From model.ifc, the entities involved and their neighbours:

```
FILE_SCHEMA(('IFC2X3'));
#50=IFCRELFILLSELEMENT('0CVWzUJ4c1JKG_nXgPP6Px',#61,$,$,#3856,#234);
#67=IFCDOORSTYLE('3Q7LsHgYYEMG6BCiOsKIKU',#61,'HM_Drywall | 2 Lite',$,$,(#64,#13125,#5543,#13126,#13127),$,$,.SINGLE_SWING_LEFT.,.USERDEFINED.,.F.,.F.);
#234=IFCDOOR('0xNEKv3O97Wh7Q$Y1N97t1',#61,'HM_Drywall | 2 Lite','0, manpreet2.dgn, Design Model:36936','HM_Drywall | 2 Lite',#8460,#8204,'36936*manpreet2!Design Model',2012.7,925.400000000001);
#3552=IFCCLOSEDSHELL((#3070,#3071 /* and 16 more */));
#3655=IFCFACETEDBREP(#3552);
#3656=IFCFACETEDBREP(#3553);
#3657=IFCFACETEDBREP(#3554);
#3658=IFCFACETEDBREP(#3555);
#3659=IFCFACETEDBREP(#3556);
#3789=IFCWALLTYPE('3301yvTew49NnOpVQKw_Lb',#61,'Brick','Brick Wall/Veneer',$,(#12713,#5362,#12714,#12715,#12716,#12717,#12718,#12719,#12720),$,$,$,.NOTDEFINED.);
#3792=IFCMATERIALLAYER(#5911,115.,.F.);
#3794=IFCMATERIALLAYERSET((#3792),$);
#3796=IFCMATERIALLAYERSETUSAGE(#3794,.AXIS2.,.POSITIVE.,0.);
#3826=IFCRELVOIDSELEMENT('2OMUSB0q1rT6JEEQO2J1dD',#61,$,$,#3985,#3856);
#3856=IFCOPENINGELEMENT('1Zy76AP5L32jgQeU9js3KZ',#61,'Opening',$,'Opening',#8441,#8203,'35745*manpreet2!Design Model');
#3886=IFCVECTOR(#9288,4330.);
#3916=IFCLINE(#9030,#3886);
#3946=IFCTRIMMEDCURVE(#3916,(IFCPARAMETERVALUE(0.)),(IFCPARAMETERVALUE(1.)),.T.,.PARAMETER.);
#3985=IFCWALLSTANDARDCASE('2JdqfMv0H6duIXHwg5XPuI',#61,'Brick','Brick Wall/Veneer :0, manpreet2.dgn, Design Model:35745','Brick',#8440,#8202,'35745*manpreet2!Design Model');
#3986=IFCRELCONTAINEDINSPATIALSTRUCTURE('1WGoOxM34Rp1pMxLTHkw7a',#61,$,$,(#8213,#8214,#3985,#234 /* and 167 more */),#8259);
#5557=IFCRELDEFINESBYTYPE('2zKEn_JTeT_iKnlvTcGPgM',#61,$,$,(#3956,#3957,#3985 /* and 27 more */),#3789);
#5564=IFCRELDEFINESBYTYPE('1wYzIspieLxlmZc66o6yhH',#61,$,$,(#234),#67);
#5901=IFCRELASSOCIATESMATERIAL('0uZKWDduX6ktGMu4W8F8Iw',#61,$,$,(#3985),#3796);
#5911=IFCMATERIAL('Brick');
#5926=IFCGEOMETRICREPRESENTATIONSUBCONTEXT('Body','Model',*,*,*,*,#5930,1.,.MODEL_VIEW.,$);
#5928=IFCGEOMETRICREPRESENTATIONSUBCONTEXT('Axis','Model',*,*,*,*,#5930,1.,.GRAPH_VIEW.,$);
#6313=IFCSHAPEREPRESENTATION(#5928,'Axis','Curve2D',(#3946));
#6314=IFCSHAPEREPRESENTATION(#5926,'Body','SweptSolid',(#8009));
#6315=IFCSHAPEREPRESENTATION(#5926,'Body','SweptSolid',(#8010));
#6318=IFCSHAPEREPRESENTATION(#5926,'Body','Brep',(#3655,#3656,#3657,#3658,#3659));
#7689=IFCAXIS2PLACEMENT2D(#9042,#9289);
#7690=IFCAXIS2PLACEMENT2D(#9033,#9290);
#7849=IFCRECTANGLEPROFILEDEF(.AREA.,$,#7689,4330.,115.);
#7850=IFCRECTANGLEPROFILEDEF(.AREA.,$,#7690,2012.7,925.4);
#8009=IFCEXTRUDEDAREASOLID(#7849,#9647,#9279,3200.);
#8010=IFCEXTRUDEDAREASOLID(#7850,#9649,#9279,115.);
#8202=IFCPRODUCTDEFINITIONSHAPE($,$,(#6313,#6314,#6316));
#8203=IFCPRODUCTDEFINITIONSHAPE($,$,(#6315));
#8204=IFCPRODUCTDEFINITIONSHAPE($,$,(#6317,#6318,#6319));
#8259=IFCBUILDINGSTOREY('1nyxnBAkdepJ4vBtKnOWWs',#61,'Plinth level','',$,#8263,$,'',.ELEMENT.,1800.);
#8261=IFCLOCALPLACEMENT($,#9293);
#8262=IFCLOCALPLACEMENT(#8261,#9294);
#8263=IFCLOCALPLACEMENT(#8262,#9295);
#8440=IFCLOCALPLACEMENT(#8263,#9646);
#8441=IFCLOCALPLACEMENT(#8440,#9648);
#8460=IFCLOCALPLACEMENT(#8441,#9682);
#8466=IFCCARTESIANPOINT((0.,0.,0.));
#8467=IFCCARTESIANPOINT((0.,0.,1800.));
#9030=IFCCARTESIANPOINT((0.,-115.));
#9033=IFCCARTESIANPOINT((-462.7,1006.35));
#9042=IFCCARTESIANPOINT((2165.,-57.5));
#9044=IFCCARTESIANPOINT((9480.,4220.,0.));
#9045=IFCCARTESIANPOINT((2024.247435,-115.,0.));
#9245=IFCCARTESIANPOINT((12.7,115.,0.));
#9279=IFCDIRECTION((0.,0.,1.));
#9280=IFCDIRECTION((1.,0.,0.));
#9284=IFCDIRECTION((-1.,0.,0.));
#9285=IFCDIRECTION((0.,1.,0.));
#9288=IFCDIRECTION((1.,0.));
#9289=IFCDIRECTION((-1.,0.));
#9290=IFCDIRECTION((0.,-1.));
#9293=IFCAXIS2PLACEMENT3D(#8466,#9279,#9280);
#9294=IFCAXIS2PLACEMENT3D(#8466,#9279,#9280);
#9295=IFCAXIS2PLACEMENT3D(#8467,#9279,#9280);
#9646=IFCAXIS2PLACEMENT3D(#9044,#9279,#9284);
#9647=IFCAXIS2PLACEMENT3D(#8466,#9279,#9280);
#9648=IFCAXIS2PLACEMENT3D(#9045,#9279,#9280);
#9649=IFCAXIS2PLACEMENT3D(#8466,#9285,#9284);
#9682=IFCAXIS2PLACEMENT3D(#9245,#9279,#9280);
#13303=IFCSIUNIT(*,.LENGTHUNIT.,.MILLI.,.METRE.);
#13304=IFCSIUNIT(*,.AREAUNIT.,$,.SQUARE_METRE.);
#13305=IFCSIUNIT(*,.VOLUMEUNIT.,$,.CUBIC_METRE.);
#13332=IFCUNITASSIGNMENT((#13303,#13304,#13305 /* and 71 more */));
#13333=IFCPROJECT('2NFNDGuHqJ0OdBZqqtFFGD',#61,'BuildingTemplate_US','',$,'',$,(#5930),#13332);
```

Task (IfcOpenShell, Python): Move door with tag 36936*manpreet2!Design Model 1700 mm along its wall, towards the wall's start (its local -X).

```python
import ifcopenshell
import ifcopenshell.api.geometry
import ifcopenshell.util.placement

model = ifcopenshell.open("model.ifc")

door = model.by_id(234)
opening = door.FillsVoids[0].RelatingOpeningElement
wall = opening.VoidsElements[0].RelatingBuildingElement

wall_matrix = ifcopenshell.util.placement.get_local_placement(wall.ObjectPlacement)
shift = wall_matrix[:3, 0] * -1700.0
before = ifcopenshell.util.placement.get_local_placement(door.ObjectPlacement)[:3, 3].copy()

# The door is placed relative to its opening, so it follows when the opening moves.
matrix = ifcopenshell.util.placement.get_local_placement(opening.ObjectPlacement)
matrix[:3, 3] += shift
ifcopenshell.api.geometry.edit_object_placement(
    model, product=opening, matrix=matrix, is_si=False, should_transform_children=True
)

after = ifcopenshell.util.placement.get_local_placement(door.ObjectPlacement)[:3, 3]
print("door moved by", (after - before).round(3) + 0.0)

model.write("model_rev.ifc")
```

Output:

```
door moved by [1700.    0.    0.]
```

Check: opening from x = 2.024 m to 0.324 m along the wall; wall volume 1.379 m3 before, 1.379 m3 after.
